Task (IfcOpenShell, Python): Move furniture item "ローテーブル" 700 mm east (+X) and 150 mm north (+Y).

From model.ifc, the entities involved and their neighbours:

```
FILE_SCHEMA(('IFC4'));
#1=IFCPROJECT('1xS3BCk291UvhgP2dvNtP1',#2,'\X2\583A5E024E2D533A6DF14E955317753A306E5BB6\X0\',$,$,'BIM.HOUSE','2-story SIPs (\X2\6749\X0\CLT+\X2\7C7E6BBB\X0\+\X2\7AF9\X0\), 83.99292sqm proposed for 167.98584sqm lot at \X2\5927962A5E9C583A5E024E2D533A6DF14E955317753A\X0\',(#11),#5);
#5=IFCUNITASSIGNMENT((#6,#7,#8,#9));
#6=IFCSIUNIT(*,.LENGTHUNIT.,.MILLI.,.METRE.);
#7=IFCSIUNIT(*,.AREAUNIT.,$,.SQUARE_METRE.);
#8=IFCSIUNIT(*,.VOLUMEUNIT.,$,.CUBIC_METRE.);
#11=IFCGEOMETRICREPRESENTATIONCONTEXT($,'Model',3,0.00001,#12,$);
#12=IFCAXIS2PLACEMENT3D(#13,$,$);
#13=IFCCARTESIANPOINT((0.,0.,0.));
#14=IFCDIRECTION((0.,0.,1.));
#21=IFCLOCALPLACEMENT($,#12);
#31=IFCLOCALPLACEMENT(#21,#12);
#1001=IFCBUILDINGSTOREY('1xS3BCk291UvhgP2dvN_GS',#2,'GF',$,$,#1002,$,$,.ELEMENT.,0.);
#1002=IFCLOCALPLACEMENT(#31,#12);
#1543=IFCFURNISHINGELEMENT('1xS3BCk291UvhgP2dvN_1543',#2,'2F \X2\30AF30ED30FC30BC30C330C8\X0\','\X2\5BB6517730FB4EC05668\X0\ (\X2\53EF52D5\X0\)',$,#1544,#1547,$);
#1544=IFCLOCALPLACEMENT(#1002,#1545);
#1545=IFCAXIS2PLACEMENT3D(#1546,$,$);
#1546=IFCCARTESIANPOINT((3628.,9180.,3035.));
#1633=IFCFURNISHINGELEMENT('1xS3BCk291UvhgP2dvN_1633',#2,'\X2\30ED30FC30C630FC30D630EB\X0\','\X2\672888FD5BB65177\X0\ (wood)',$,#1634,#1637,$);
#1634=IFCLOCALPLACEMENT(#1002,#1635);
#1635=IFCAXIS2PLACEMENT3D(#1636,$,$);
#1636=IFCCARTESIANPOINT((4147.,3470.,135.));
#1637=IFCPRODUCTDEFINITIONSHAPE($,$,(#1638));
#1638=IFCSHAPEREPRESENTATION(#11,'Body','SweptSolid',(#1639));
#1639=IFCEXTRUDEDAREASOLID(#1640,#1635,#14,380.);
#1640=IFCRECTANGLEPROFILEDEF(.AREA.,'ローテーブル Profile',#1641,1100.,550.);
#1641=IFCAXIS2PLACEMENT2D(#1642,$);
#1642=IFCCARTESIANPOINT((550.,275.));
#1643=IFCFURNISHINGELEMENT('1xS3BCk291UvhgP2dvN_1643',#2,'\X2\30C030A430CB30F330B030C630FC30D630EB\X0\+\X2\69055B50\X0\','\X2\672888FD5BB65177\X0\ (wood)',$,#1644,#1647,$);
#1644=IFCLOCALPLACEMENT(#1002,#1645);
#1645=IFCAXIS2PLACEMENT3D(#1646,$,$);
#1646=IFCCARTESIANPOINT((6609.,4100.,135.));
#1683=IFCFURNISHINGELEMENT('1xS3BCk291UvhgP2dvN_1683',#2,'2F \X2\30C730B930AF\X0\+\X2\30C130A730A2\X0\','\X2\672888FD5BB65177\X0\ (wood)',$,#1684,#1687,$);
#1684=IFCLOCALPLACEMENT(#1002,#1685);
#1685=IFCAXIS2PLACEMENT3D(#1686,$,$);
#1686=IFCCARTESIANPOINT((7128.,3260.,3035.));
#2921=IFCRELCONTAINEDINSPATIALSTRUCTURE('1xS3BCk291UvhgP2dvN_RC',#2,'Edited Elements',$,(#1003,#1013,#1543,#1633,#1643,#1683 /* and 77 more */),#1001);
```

```python
import ifcopenshell
import ifcopenshell.api.geometry
import ifcopenshell.util.placement

model = ifcopenshell.open("model.ifc")

item = model.by_id(1633)
matrix = ifcopenshell.util.placement.get_local_placement(item.ObjectPlacement)
matrix[0, 3] += 700.0
matrix[1, 3] += 150.0
ifcopenshell.api.geometry.edit_object_placement(model, product=item, matrix=matrix, is_si=False)

print(ifcopenshell.util.placement.get_local_placement(item.ObjectPlacement).round(3) + 0.0)

model.write("model_edited.ifc")
```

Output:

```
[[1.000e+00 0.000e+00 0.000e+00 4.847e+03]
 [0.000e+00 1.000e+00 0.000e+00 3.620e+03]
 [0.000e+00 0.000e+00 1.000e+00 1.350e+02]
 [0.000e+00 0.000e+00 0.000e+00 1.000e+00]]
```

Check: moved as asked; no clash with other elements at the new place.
